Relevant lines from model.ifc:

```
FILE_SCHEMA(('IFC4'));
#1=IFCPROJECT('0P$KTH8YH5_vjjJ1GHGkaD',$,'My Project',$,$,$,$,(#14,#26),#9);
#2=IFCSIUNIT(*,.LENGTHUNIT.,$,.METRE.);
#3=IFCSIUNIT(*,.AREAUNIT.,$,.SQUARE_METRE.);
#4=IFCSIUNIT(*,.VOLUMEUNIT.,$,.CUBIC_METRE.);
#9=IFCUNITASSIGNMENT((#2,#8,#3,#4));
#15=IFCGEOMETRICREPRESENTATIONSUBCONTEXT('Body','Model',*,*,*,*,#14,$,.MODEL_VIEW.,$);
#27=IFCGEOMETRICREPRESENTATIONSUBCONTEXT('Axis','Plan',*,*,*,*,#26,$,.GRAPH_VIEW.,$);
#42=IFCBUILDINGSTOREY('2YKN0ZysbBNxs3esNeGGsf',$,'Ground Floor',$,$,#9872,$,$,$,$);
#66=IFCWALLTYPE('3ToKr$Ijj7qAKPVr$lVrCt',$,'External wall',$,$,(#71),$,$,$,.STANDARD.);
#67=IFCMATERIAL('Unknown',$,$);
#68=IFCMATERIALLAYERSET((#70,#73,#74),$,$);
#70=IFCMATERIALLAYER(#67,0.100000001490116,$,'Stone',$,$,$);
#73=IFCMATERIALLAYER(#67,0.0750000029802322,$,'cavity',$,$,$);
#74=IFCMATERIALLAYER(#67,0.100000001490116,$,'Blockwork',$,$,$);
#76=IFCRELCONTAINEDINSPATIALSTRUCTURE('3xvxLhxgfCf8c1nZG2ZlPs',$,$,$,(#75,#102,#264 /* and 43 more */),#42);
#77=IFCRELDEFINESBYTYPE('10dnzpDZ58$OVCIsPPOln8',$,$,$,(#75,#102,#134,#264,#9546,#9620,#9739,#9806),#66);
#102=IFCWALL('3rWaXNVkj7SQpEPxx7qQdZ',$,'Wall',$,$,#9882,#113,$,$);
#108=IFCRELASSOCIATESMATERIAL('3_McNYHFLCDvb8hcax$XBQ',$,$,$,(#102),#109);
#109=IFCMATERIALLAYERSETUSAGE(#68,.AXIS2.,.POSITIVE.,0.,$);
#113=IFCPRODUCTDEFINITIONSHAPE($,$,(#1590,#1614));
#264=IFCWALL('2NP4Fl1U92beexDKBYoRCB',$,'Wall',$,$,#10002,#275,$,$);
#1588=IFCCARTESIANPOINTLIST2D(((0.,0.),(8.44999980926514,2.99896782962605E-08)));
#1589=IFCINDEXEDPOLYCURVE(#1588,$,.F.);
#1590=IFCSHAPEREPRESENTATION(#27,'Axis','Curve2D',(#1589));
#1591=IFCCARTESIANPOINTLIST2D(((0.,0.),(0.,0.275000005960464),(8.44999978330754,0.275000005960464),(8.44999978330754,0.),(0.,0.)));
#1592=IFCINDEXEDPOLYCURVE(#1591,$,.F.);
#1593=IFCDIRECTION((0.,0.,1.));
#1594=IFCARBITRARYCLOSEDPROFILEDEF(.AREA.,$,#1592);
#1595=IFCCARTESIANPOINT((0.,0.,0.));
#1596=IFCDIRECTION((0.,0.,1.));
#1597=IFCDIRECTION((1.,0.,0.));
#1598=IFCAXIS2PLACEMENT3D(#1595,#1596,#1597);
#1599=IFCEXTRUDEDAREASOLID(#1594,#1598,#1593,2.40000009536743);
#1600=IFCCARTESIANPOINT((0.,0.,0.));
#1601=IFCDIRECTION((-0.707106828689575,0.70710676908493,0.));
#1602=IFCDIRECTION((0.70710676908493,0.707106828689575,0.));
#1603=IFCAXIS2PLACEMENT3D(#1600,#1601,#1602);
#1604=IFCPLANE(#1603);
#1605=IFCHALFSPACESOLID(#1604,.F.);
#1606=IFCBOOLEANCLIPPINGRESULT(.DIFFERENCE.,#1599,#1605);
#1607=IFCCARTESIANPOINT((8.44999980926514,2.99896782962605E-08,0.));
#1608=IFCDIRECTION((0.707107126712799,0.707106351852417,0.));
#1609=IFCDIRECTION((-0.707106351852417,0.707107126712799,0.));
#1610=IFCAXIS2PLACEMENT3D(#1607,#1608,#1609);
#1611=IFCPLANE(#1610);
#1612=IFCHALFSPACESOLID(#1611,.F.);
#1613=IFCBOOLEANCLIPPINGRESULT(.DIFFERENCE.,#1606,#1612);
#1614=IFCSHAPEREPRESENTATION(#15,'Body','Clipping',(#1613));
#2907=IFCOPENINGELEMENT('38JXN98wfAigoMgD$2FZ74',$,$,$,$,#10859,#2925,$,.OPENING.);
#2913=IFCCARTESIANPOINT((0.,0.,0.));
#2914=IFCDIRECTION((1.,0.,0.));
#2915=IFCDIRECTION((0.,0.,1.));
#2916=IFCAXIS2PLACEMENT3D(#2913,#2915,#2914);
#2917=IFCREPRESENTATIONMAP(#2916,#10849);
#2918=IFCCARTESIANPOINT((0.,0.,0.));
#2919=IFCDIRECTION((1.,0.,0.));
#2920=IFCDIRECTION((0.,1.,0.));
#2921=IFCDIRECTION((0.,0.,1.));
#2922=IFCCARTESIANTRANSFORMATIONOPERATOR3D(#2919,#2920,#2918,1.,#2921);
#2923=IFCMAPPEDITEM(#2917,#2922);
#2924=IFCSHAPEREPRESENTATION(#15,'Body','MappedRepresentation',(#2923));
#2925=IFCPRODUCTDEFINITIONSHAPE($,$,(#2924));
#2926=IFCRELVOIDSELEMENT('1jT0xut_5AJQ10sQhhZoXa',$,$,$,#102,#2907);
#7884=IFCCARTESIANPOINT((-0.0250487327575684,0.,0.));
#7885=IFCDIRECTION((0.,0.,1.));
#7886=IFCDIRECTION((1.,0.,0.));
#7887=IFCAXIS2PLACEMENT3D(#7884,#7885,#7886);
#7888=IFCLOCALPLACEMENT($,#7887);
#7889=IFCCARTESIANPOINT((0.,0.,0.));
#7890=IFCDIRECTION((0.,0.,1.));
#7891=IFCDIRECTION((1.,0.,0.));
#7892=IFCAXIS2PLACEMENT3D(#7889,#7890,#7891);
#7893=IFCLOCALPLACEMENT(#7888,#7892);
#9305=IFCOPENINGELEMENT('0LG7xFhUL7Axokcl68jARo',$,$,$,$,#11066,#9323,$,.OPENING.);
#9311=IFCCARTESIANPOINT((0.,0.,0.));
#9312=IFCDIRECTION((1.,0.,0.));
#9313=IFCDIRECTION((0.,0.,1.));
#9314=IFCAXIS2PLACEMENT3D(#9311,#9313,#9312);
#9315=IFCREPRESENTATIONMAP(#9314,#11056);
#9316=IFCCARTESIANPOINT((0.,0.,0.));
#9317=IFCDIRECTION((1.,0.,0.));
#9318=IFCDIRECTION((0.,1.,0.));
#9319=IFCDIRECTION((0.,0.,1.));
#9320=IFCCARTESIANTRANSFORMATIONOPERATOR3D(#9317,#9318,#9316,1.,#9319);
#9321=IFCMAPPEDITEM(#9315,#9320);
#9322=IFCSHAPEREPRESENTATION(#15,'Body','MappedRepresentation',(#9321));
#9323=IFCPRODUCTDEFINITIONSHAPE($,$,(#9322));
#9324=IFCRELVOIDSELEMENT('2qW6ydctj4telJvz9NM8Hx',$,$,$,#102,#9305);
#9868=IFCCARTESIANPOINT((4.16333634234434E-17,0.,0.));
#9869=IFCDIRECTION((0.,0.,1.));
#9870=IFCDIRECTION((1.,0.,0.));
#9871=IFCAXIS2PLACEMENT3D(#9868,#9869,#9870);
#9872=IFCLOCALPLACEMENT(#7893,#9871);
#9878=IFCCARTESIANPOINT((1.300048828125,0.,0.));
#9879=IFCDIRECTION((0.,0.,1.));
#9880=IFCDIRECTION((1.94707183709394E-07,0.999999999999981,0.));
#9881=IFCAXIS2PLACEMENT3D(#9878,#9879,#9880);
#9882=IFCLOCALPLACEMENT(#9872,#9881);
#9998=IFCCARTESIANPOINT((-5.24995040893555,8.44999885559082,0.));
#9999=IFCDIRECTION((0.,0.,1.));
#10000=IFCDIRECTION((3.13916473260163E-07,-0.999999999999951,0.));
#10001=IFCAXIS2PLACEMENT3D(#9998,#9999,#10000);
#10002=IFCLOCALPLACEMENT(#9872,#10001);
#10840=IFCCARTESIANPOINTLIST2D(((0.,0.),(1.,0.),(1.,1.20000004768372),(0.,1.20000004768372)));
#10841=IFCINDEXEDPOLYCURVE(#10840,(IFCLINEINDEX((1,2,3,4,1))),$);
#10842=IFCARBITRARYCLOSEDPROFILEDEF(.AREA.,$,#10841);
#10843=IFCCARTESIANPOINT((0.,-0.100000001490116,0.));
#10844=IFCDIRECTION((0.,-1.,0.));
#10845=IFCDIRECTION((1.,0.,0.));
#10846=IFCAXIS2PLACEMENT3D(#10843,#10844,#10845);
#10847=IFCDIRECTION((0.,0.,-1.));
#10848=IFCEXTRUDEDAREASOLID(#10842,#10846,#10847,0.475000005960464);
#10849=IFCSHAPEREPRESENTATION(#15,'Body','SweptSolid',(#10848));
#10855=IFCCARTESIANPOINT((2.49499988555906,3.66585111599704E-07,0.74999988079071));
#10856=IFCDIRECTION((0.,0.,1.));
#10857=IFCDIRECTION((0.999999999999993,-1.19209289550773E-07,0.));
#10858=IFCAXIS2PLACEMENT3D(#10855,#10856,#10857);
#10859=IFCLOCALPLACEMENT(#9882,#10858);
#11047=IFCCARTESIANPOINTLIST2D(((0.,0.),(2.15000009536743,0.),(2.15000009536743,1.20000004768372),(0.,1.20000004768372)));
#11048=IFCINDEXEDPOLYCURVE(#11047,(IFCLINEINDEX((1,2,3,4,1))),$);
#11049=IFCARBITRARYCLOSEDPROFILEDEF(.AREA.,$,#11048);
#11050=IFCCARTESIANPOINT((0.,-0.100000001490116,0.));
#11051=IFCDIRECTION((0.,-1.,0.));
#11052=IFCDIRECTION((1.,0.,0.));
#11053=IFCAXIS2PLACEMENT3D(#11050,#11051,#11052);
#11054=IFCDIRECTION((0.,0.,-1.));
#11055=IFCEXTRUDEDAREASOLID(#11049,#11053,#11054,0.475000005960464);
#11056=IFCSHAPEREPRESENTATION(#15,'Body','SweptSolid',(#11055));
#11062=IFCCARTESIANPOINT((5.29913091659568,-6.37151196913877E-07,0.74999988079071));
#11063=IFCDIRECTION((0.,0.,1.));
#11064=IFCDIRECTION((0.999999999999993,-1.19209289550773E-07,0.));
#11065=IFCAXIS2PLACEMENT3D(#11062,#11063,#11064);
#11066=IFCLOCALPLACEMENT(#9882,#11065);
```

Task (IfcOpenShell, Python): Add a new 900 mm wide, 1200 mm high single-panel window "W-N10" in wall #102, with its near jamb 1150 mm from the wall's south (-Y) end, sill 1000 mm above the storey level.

```python
import numpy as np
import ifcopenshell
import ifcopenshell.api.feature
import ifcopenshell.api.geometry
import ifcopenshell.api.root
import ifcopenshell.api.spatial
import ifcopenshell.geom
import ifcopenshell.util.element
import ifcopenshell.util.placement
import ifcopenshell.util.representation
import ifcopenshell.util.shape
import ifcopenshell.util.unit

model = ifcopenshell.open("model.ifc")
unit_scale = ifcopenshell.util.unit.calculate_unit_scale(model)
settings = ifcopenshell.geom.settings()


def volume(element):
    """Net volume in cubic metres, openings subtracted."""
    shape = ifcopenshell.geom.create_shape(settings, element)
    return ifcopenshell.util.shape.get_volume(shape.geometry)


wall = model.by_guid("3rWaXNVkj7SQpEPxx7qQdZ")
storey = ifcopenshell.util.element.get_container(wall, ifc_class="IfcBuildingStorey")
context = ifcopenshell.util.representation.get_context(model, "Model", "Body", "MODEL_VIEW")
before = volume(wall)

width, height, from_end, sill = 0.9, 1.2, 1.15, 1  # metres

# The wall runs along its own X axis, and the end named is its -X end.
wall_shape = ifcopenshell.geom.create_shape(settings, wall)
x, y, z = ifcopenshell.util.shape.get_vertices(wall_shape.geometry).T
start = x.min() + from_end
face, thickness = float(y.min()), float(y.max() - y.min())
wall_matrix = ifcopenshell.util.placement.get_local_placement(wall.ObjectPlacement)
level = ifcopenshell.util.placement.get_local_placement(storey.ObjectPlacement)[2, 3]


def in_wall(x, y):
    """Placement at x, y metres in the wall's axes, at sill height."""
    matrix = wall_matrix.copy()
    matrix[:, 3] = wall_matrix @ np.array([x / unit_scale, y / unit_scale, 0.0, 1.0])
    matrix[2, 3] = level + sill / unit_scale
    return matrix


# Opening: a box that overshoots both wall faces by 50 mm.
opening = ifcopenshell.api.root.create_entity(model, ifc_class="IfcOpeningElement", predefined_type="OPENING")
box = ifcopenshell.api.geometry.add_wall_representation(
    model, context=context, length=width, height=height, thickness=thickness + 0.1
)
ifcopenshell.api.geometry.assign_representation(model, product=opening, representation=box)
ifcopenshell.api.geometry.edit_object_placement(model, product=opening, matrix=in_wall(start, face - 0.05), is_si=False)
ifcopenshell.api.feature.add_feature(model, feature=opening, element=wall)

window = ifcopenshell.api.root.create_entity(model, ifc_class="IfcWindow", name="W-N10", predefined_type="WINDOW")
window.OverallWidth, window.OverallHeight = width / unit_scale, height / unit_scale
window.PartitioningType = "SINGLE_PANEL"
body = ifcopenshell.api.geometry.add_window_representation(
    model,
    context=context,
    overall_width=window.OverallWidth,
    overall_height=window.OverallHeight,
    partition_type="SINGLE_PANEL",
)
ifcopenshell.api.geometry.assign_representation(model, product=window, representation=body)
ifcopenshell.api.spatial.assign_container(model, products=[window], relating_structure=storey)
ifcopenshell.api.feature.add_filling(model, opening=opening, element=window)

# Centre the window in the wall's thickness.
ifcopenshell.api.geometry.edit_object_placement(model, product=window, matrix=in_wall(start, face), is_si=False)
window_shape = ifcopenshell.geom.create_shape(settings, window)
depth = ifcopenshell.util.shape.get_vertices(window_shape.geometry)[:, 1]
offset = face + thickness / 2 - (depth.min() + depth.max()) / 2
ifcopenshell.api.geometry.edit_object_placement(model, product=window, matrix=in_wall(start, offset), is_si=False)

after = volume(wall)

print(f"wall volume {before:.3f} -> {after:.3f} m3")

model.write("model_v2.ifc")
```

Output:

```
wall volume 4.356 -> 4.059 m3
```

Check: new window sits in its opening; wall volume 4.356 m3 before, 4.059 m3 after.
